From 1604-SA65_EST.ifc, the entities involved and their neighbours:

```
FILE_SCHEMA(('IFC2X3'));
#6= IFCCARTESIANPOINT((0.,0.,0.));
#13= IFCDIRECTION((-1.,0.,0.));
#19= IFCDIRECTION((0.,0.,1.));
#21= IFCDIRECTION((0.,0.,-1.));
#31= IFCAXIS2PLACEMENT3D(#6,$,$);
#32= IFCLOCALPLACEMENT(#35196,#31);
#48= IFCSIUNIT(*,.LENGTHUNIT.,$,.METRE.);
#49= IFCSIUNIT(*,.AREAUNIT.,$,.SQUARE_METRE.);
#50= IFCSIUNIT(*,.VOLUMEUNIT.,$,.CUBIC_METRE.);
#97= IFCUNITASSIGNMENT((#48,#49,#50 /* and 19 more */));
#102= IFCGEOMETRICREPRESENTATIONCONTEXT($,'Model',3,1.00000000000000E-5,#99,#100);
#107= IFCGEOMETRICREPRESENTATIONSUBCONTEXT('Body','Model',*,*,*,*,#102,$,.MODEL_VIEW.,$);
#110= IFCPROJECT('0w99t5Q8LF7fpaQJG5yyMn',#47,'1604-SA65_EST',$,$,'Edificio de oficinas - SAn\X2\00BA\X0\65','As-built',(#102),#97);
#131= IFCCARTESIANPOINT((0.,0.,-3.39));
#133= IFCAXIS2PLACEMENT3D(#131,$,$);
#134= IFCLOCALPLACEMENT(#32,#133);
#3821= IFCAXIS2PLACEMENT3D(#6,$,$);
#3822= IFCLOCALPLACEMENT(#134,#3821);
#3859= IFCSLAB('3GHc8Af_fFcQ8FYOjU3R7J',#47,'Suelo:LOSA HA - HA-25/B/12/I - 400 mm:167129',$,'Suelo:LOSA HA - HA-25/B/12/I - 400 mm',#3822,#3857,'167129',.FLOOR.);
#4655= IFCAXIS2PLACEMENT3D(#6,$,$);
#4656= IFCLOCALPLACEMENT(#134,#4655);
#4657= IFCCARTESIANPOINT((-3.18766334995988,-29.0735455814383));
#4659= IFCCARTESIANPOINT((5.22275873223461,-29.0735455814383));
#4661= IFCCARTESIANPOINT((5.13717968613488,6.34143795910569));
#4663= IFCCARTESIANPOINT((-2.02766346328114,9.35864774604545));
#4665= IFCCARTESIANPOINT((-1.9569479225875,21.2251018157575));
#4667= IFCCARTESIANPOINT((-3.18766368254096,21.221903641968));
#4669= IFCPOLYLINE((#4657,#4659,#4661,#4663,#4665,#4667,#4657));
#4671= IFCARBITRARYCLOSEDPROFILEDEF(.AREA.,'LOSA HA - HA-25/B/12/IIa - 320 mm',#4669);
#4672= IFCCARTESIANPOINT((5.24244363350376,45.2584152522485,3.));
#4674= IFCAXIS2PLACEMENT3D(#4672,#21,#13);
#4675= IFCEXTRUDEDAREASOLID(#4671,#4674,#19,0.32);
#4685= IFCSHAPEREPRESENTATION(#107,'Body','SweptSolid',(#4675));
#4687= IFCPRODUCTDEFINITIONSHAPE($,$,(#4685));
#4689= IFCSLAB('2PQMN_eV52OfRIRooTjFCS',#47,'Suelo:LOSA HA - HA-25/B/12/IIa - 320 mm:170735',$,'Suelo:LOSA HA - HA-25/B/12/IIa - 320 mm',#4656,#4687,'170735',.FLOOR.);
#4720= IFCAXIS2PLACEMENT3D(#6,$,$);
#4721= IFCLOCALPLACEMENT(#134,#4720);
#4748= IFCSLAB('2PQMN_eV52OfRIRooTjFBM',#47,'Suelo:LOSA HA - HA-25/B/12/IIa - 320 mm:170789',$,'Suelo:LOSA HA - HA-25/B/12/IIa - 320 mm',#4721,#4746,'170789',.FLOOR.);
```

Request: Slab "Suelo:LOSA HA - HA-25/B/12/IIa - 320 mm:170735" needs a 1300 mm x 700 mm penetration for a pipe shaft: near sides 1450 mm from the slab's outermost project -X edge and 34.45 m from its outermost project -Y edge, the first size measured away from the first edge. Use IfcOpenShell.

```python
import numpy as np
import ifcopenshell
import ifcopenshell.api.feature
import ifcopenshell.api.geometry
import ifcopenshell.api.root
import ifcopenshell.geom
import ifcopenshell.util.placement
import ifcopenshell.util.representation
import ifcopenshell.util.shape
import ifcopenshell.util.unit

model = ifcopenshell.open("1604-SA65_EST.ifc")
unit_scale = ifcopenshell.util.unit.calculate_unit_scale(model)
settings = ifcopenshell.geom.settings()


def volume(element):
    """Net volume in cubic metres, openings subtracted."""
    shape = ifcopenshell.geom.create_shape(settings, element)
    return ifcopenshell.util.shape.get_volume(shape.geometry)


slab = model.by_guid("2PQMN_eV52OfRIRooTjFCS")
before = volume(slab)

# Extent in the slab's own axes, in metres. The edges named are its -X and -Y sides.
slab_shape = ifcopenshell.geom.create_shape(settings, slab)
vertices = ifcopenshell.util.shape.get_vertices(slab_shape.geometry)
x_min, y_min, bottom = vertices.min(axis=0)
top = vertices[:, 2].max()

opening = ifcopenshell.api.root.create_entity(model, ifc_class="IfcOpeningElement", name="Pipe shaft opening")
context = ifcopenshell.util.representation.get_context(model, "Model", "Body", "MODEL_VIEW")
width, depth = 1.3, 0.7
outline = [(0.0, 0.0), (width, 0.0), (width, depth), (0.0, depth), (0.0, 0.0)]
# Overshoot both faces by 50 mm so the cut is clean.
shape = ifcopenshell.api.geometry.add_slab_representation(
    model, context=context, depth=top - bottom + 0.1, polyline=outline
)
ifcopenshell.api.geometry.assign_representation(model, product=opening, representation=shape)

matrix = ifcopenshell.util.placement.get_local_placement(slab.ObjectPlacement)
matrix[:, 3] = matrix @ np.append(np.array([x_min + 1.45, y_min + 34.45, bottom - 0.05]) / unit_scale, 1.0)
ifcopenshell.api.geometry.edit_object_placement(model, product=opening, matrix=matrix, is_si=False)
ifcopenshell.api.feature.add_feature(model, feature=opening, element=slab)

after = volume(slab)

print(f"slab volume {before:.3f} -> {after:.3f} m3")

model.write("1604-SA65_EST_updated.ifc")
```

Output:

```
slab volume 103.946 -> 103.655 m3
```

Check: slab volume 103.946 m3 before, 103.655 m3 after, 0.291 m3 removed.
